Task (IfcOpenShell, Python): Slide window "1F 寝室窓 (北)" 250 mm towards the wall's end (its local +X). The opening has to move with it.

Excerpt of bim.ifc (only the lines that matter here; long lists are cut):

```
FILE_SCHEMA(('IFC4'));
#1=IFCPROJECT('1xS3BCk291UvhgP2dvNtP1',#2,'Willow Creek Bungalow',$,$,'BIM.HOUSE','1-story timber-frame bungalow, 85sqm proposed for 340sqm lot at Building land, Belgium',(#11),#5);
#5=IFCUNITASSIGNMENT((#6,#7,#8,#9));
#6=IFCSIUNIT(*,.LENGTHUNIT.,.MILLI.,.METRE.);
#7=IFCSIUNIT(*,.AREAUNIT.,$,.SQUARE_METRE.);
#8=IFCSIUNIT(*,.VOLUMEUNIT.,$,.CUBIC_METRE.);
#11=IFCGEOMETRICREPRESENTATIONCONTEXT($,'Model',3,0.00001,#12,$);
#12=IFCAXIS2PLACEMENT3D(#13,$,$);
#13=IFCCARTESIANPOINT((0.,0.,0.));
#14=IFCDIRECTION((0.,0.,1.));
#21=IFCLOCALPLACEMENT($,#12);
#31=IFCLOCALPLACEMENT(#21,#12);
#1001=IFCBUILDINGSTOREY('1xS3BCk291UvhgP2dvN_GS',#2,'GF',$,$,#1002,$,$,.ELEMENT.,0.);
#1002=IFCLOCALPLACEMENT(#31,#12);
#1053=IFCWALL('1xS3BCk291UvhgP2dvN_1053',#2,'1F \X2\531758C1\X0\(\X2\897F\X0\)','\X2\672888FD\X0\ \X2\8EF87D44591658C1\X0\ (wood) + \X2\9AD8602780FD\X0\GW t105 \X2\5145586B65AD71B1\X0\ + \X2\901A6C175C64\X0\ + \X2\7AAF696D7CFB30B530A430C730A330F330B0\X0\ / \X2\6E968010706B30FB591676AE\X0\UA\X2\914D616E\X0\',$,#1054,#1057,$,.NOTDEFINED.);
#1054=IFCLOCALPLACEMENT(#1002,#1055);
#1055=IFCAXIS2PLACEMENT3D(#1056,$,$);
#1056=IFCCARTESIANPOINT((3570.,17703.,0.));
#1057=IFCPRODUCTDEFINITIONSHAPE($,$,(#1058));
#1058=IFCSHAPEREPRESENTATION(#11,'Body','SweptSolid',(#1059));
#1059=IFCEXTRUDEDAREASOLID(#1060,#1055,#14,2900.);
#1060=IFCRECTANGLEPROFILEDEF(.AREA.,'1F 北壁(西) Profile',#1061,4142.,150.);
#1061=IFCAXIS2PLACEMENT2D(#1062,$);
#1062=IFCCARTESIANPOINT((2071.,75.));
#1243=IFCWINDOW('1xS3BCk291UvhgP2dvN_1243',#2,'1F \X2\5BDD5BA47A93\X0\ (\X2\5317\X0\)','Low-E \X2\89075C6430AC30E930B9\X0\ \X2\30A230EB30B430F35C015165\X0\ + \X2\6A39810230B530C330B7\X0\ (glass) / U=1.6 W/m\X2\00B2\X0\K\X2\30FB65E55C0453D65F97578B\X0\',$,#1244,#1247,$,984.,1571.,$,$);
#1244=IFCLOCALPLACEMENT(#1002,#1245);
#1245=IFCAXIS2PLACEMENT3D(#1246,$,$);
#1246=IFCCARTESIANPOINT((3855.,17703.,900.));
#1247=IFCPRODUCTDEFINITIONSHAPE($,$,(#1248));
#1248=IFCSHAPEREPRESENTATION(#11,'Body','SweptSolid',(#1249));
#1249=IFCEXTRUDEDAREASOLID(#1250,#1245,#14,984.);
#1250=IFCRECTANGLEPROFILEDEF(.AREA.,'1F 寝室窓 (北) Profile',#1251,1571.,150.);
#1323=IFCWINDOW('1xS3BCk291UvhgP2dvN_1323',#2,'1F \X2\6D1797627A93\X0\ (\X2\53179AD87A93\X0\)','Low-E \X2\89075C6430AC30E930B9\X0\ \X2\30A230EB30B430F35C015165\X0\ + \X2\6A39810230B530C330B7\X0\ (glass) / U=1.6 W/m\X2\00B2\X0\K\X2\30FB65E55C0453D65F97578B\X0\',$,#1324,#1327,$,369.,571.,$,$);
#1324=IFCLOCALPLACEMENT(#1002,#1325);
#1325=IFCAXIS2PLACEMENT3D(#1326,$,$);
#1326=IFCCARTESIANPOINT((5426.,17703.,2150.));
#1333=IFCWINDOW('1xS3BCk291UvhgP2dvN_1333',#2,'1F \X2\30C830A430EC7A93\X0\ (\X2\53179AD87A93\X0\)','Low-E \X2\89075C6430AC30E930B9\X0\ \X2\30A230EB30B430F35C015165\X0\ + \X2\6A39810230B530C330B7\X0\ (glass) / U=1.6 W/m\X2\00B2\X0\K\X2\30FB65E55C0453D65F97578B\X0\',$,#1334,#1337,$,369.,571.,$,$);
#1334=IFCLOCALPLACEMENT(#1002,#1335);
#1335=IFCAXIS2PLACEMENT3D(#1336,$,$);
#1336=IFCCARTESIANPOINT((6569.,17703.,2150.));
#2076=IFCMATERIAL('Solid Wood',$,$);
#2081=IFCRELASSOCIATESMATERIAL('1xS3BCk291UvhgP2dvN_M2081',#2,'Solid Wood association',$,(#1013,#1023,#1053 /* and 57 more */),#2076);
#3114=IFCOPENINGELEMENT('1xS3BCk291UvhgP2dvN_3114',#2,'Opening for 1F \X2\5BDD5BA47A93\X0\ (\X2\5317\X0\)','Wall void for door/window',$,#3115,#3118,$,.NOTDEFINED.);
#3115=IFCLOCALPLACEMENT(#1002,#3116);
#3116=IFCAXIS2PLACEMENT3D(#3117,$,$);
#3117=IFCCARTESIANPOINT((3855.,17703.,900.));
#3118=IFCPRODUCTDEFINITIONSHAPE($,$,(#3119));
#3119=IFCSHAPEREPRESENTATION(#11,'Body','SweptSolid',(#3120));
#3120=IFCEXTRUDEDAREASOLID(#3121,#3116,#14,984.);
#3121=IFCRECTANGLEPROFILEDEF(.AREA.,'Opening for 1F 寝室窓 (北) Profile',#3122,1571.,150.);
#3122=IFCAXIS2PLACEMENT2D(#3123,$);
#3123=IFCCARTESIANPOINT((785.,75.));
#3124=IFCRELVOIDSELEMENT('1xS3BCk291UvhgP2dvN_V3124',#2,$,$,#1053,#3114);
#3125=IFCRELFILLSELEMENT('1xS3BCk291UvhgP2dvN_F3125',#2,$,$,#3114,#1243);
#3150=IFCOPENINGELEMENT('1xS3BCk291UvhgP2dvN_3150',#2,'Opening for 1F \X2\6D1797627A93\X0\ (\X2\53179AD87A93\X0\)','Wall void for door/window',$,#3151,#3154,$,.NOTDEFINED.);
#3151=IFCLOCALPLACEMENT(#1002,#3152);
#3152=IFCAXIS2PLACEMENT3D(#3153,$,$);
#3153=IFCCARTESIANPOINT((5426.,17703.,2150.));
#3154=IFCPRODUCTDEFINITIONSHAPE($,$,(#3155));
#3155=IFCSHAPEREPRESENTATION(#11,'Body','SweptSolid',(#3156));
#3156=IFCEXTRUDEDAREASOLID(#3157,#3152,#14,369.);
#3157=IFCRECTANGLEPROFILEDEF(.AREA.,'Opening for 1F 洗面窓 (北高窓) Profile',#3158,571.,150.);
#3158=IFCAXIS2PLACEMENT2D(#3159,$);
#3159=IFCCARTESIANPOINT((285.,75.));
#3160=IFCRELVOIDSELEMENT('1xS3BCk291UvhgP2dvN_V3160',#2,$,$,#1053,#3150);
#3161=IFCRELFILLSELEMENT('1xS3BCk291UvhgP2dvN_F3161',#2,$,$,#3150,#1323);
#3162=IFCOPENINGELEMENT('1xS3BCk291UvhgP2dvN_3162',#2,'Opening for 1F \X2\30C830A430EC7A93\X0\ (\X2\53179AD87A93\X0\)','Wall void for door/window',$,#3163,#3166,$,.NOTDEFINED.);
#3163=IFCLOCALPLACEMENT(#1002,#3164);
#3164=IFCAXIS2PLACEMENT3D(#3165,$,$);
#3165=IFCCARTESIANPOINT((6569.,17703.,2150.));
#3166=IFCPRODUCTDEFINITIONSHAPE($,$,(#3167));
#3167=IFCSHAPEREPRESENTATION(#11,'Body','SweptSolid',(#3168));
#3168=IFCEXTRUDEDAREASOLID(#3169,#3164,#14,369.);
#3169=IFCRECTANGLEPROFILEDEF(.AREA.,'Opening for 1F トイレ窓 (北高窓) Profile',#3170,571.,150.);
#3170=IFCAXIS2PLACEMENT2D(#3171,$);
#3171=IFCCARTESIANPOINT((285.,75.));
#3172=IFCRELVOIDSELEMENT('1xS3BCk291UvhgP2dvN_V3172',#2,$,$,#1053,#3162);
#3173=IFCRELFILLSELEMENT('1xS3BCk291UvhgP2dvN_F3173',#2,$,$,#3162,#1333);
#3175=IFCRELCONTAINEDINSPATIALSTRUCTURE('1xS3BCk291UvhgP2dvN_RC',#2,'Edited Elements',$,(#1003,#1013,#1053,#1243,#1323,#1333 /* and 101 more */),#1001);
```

```python
import ifcopenshell
import ifcopenshell.api.geometry
import ifcopenshell.util.placement
import ifcopenshell.util.unit

model = ifcopenshell.open("bim.ifc")
unit_scale = ifcopenshell.util.unit.calculate_unit_scale(model)

window = model.by_guid("1xS3BCk291UvhgP2dvN_1243")
opening = window.FillsVoids[0].RelatingOpeningElement
wall = opening.VoidsElements[0].RelatingBuildingElement

wall_matrix = ifcopenshell.util.placement.get_local_placement(wall.ObjectPlacement)
shift = wall_matrix[:3, 0] * 0.25 / unit_scale
before = ifcopenshell.util.placement.get_local_placement(window.ObjectPlacement)[:3, 3].copy()

# The window is not placed relative to its opening, so move both.
for product in (opening, window):
    matrix = ifcopenshell.util.placement.get_local_placement(product.ObjectPlacement)
    matrix[:3, 3] += shift
    ifcopenshell.api.geometry.edit_object_placement(model, product=product, matrix=matrix, is_si=False)

after = ifcopenshell.util.placement.get_local_placement(window.ObjectPlacement)[:3, 3]
print("window moved by", (after - before).round(3) + 0.0)

model.write("bim_edited.ifc")
```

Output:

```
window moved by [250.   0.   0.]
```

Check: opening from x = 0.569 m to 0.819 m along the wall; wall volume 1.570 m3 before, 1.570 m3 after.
